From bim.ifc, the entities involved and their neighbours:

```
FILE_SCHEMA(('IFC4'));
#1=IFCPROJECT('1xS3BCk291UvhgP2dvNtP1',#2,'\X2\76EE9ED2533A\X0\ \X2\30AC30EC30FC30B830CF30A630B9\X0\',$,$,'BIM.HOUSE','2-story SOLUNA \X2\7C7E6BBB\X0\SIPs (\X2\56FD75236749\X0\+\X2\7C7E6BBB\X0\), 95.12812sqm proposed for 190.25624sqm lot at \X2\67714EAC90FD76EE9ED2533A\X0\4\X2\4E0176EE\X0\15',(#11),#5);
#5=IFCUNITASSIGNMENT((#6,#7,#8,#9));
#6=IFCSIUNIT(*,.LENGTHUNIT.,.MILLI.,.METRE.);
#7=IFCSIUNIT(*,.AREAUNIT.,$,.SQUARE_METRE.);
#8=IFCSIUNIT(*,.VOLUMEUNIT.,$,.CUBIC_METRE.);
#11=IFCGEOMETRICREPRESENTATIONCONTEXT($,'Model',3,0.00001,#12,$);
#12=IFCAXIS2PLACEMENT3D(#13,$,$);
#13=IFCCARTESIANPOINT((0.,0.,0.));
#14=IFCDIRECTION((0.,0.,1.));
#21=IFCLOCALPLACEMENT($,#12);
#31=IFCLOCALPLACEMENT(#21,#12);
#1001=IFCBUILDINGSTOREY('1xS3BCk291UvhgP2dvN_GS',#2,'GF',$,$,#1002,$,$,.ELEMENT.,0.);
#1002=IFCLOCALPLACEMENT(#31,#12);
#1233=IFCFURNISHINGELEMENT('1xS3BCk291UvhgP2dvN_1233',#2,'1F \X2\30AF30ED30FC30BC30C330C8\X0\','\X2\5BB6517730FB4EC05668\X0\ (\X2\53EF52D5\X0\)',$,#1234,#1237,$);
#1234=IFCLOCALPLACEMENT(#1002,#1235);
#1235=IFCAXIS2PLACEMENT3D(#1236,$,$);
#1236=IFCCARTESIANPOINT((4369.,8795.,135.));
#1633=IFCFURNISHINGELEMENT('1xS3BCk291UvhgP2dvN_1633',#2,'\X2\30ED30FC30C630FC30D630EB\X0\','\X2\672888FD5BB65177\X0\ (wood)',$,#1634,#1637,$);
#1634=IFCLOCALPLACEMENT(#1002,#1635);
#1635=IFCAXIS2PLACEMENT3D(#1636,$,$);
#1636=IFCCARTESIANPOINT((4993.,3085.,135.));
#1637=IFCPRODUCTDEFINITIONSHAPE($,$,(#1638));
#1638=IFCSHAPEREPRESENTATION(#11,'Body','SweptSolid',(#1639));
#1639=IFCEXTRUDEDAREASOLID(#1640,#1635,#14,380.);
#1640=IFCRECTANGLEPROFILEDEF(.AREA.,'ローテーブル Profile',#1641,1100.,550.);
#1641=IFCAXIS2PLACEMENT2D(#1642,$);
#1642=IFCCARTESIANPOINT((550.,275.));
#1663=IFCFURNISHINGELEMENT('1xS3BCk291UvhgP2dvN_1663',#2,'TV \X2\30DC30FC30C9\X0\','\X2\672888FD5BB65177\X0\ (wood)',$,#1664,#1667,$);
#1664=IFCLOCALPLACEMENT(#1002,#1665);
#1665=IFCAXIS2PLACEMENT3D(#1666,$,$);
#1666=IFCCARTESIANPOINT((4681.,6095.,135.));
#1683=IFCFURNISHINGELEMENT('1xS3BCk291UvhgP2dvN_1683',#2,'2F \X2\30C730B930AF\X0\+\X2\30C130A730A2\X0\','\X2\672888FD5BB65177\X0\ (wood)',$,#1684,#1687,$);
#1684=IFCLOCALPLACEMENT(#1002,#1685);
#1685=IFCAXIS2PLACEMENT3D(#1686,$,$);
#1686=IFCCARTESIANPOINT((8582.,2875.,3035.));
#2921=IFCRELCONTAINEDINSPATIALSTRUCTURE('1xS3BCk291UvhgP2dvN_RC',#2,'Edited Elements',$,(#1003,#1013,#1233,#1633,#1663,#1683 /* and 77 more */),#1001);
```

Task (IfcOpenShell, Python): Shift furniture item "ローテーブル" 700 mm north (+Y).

```python
import ifcopenshell
import ifcopenshell.api.geometry
import ifcopenshell.util.placement
import ifcopenshell.util.unit

model = ifcopenshell.open("bim.ifc")
unit_scale = ifcopenshell.util.unit.calculate_unit_scale(model)

item = model.by_id(1633)
matrix = ifcopenshell.util.placement.get_local_placement(item.ObjectPlacement)
matrix[1, 3] += 0.7 / unit_scale
ifcopenshell.api.geometry.edit_object_placement(model, product=item, matrix=matrix, is_si=False)

print(ifcopenshell.util.placement.get_local_placement(item.ObjectPlacement).round(3) + 0.0)

model.write("bim-out.ifc")
```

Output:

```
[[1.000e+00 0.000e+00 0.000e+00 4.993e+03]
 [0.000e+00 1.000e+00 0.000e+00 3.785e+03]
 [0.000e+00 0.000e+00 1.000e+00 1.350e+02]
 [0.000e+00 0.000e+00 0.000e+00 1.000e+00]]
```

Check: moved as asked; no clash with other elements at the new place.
